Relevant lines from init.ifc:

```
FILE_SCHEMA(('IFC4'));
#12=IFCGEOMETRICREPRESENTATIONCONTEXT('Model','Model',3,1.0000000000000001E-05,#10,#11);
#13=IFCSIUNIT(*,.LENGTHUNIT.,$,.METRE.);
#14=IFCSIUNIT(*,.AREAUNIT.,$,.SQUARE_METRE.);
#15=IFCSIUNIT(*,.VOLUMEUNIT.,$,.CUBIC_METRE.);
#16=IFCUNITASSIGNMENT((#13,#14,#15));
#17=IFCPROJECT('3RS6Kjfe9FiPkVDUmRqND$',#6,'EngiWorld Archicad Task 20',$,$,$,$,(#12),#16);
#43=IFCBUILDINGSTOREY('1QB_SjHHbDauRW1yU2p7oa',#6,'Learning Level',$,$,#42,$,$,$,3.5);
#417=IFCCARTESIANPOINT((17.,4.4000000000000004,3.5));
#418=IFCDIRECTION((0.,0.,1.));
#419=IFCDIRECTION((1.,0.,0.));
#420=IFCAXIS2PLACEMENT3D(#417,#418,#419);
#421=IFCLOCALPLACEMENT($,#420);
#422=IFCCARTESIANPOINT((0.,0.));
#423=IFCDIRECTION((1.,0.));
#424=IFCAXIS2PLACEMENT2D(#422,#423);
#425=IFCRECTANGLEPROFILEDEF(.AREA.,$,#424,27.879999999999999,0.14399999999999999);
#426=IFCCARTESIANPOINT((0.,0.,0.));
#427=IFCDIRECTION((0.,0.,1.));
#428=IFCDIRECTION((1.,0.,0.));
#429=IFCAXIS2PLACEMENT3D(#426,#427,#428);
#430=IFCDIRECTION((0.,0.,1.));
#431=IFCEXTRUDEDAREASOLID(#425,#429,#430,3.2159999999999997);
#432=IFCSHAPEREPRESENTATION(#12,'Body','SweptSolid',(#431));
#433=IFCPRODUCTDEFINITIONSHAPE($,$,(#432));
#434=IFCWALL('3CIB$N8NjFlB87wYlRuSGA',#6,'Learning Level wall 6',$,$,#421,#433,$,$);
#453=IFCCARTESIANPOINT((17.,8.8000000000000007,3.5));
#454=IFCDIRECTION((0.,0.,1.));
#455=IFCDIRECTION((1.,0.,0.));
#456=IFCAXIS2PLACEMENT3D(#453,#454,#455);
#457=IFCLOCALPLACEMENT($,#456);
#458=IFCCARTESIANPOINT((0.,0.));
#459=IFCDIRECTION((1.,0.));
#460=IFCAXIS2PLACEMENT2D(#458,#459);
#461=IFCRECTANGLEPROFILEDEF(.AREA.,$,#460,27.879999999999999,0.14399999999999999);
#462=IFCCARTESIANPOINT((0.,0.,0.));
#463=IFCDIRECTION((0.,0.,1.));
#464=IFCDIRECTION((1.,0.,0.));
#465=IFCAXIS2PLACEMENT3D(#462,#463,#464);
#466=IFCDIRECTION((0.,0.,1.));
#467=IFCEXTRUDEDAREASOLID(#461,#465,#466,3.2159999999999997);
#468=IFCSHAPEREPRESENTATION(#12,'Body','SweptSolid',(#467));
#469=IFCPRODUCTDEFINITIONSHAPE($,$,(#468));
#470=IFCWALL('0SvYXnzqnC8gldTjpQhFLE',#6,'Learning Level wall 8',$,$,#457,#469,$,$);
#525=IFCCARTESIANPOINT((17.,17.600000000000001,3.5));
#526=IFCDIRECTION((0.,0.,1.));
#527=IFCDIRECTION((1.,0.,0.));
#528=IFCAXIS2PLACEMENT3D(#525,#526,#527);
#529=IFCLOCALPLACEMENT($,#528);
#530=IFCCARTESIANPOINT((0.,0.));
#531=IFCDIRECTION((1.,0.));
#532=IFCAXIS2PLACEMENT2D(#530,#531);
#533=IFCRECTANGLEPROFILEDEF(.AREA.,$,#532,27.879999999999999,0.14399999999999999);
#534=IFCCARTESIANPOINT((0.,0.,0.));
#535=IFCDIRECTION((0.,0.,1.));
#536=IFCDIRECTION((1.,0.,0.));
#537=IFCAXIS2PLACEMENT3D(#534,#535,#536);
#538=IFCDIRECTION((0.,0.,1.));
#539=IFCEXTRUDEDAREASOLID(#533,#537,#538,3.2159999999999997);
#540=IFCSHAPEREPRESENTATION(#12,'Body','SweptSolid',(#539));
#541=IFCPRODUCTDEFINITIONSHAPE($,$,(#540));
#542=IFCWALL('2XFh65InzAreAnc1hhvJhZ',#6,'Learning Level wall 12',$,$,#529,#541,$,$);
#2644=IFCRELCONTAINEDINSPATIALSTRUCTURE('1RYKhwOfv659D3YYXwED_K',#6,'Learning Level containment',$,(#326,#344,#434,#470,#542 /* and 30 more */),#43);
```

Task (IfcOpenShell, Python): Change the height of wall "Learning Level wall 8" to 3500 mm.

```python
import ifcopenshell
import ifcopenshell.geom
import ifcopenshell.util.shape
import ifcopenshell.util.unit

model = ifcopenshell.open("init.ifc")
unit_scale = ifcopenshell.util.unit.calculate_unit_scale(model)
settings = ifcopenshell.geom.settings()


def volume(element):
    """Net volume in cubic metres, openings subtracted."""
    shape = ifcopenshell.geom.create_shape(settings, element)
    return ifcopenshell.util.shape.get_volume(shape.geometry)


wall = model.by_id(470)
before = volume(wall)

body = next(r for r in wall.Representation.Representations if r.RepresentationIdentifier == "Body")
solid = body.Items[0]
old_height = solid.Depth
solid.Depth = 3.5 / unit_scale
after = volume(wall)

print(f"height {old_height:g} -> {solid.Depth:g}, volume {before:.3f} -> {after:.3f} m3")

model.write("init_updated.ifc")
```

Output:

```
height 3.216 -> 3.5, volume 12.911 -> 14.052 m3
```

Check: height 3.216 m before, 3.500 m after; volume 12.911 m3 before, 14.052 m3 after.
